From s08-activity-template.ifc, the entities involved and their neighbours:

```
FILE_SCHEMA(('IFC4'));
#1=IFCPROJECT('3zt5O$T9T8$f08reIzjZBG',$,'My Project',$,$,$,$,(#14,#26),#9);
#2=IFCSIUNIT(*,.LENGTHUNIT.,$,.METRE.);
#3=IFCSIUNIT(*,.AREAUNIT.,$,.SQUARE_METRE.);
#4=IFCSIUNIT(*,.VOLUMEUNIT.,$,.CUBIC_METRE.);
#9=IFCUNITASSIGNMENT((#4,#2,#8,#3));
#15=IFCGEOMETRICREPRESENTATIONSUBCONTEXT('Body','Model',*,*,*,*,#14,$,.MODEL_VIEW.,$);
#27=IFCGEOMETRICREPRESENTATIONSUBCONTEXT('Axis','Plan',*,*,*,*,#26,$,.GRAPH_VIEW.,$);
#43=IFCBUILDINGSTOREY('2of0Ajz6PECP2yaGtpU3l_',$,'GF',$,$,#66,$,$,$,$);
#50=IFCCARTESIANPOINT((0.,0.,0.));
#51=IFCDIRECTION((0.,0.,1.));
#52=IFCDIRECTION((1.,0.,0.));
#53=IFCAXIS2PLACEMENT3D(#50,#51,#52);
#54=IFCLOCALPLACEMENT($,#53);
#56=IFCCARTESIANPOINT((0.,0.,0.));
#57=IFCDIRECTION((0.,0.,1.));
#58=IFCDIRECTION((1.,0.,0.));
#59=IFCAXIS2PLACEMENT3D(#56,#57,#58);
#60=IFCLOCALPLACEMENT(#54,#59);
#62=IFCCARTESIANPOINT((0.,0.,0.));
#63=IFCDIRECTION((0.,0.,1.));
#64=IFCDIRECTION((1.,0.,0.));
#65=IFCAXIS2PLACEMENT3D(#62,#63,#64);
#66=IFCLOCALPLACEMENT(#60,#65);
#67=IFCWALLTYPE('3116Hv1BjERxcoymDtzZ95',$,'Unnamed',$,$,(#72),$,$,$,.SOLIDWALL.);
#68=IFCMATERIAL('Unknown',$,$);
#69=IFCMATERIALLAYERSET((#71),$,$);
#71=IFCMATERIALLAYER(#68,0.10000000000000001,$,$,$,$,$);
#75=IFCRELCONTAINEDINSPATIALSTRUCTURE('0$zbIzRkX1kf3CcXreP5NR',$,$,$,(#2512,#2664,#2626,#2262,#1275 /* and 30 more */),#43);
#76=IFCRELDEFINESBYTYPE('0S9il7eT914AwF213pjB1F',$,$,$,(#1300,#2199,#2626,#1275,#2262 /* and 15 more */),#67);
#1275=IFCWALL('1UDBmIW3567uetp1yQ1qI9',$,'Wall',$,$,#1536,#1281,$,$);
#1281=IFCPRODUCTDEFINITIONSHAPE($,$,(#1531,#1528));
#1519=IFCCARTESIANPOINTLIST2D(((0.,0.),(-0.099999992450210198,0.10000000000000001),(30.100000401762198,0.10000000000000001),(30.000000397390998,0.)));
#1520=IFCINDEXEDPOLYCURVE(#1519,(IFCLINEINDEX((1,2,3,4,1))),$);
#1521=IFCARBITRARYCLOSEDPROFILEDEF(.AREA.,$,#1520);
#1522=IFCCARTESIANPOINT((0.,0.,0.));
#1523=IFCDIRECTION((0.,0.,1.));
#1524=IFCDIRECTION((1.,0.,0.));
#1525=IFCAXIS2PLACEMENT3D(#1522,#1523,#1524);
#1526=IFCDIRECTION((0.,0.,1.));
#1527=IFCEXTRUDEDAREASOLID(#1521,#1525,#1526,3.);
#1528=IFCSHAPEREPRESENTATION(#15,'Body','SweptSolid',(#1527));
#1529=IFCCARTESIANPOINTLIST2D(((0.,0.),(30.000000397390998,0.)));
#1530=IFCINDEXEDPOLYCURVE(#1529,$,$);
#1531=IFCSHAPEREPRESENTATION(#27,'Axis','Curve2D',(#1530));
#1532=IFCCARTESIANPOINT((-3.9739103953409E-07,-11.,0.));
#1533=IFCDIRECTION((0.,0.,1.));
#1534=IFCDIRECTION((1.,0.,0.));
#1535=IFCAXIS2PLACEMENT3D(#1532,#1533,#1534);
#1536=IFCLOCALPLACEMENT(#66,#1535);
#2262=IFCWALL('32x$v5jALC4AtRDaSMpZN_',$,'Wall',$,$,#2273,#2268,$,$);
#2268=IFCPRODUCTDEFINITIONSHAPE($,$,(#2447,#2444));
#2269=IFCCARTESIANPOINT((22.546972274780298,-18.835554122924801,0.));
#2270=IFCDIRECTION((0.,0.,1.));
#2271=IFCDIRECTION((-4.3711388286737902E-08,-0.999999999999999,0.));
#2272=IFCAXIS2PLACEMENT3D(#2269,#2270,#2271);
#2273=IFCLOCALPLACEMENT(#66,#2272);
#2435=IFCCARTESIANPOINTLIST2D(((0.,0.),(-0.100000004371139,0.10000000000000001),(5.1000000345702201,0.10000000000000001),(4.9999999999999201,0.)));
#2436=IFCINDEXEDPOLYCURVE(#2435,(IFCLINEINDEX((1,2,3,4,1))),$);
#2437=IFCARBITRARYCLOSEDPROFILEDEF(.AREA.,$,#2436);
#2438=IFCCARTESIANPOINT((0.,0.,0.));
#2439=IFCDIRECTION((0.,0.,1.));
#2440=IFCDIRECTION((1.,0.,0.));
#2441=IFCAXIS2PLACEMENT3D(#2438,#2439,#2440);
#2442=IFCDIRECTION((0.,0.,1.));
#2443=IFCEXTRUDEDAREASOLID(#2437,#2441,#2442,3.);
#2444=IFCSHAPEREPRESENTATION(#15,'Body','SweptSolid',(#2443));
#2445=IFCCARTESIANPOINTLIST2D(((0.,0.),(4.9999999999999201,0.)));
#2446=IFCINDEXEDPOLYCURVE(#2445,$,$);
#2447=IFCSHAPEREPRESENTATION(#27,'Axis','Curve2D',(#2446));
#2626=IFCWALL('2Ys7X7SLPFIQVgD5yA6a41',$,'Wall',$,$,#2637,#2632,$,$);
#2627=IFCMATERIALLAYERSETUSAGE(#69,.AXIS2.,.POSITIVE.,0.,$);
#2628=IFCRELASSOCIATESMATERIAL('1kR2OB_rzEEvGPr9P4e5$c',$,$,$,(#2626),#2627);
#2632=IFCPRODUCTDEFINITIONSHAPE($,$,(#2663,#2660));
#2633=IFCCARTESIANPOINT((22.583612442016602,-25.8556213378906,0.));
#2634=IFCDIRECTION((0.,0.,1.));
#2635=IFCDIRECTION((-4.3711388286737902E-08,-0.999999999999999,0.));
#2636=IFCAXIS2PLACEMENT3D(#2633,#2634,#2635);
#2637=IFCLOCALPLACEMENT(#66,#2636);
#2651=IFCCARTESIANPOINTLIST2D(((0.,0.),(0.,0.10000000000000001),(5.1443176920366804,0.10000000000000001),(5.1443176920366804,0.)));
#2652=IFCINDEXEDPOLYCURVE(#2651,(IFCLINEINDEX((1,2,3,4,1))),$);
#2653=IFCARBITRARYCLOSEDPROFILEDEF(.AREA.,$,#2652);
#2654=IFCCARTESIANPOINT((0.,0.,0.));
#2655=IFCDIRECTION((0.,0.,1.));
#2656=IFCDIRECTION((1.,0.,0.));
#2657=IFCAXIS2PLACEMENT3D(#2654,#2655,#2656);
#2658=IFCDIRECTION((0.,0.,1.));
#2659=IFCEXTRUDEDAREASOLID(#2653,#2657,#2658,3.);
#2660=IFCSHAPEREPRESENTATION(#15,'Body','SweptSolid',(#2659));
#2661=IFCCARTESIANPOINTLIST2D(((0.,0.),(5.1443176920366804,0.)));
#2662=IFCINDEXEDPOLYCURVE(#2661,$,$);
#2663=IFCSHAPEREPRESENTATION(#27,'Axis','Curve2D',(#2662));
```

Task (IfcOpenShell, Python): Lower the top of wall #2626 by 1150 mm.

```python
import ifcopenshell
import ifcopenshell.geom
import ifcopenshell.util.representation
import ifcopenshell.util.shape

model = ifcopenshell.open("s08-activity-template.ifc")
settings = ifcopenshell.geom.settings()


def volume(element):
    """Net volume in cubic metres, openings subtracted."""
    shape = ifcopenshell.geom.create_shape(settings, element)
    return ifcopenshell.util.shape.get_volume(shape.geometry)


wall = model.by_guid("2Ys7X7SLPFIQVgD5yA6a41")
before = volume(wall)

body = ifcopenshell.util.representation.get_representation(wall, "Model", "Body")
solid = body.Items[0]
old_height = solid.Depth
solid.Depth -= 1.15
after = volume(wall)

print(f"height {old_height:g} -> {solid.Depth:g}, volume {before:.3f} -> {after:.3f} m3")

model.write("s08-activity-template_updated.ifc")
```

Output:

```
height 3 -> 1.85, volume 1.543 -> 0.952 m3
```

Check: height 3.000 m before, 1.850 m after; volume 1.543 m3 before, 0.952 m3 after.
